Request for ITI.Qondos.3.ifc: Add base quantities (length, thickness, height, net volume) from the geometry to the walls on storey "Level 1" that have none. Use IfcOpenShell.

First a look at what the model holds.

```python
import ifcopenshell
import ifcopenshell.util.element
import ifcopenshell.util.unit

model = ifcopenshell.open("ITI.Qondos.3.ifc")
print(model.schema)
for unit_type in ("LENGTHUNIT", "AREAUNIT", "VOLUMEUNIT"):
    print(unit_type, ifcopenshell.util.unit.calculate_unit_scale(model, unit_type))
storey = next(s for s in model.by_type("IfcBuildingStorey") if s.Name == "Level 1")
walls = [e for e in ifcopenshell.util.element.get_decomposition(storey) if e.is_a("IfcWall")]
for e in sorted(walls, key=lambda e: e.id()):
    print(e.id(), e.is_a(), e.Name, list(ifcopenshell.util.element.get_psets(e, qtos_only=True)), sep=" | ")
```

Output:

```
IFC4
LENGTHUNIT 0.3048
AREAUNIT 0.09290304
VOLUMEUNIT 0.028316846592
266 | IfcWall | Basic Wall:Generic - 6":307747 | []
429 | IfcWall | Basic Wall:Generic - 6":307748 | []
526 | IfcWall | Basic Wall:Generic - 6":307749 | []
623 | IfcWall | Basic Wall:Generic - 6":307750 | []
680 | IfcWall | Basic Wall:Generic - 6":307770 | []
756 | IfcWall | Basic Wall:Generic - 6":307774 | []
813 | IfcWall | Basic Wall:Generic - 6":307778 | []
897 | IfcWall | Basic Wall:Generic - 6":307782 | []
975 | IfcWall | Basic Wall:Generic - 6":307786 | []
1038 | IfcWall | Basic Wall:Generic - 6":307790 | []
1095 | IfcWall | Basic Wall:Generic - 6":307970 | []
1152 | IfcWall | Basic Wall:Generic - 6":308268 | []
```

```python
import ifcopenshell
import ifcopenshell.api.pset
import ifcopenshell.geom
import ifcopenshell.util.element
import ifcopenshell.util.shape
import ifcopenshell.util.unit

model = ifcopenshell.open("ITI.Qondos.3.ifc")
unit_scale = ifcopenshell.util.unit.calculate_unit_scale(model)
volume_scale = ifcopenshell.util.unit.calculate_unit_scale(model, "VOLUMEUNIT")
settings = ifcopenshell.geom.settings()

storey = next(s for s in model.by_type("IfcBuildingStorey") if s.Name == "Level 1")
walls = [e for e in ifcopenshell.util.element.get_decomposition(storey) if e.is_a("IfcWall")]

for e in sorted(walls, key=lambda e: e.id()):
    if ifcopenshell.util.element.get_psets(e, qtos_only=True, should_inherit=False):
        continue
    # Geometry comes back in metres, in the element's own axes.
    shape = ifcopenshell.geom.create_shape(settings, e)
    values = {
        "Length": ifcopenshell.util.shape.get_x(shape.geometry) / unit_scale,
        "Width": ifcopenshell.util.shape.get_y(shape.geometry) / unit_scale,
        "Height": ifcopenshell.util.shape.get_z(shape.geometry) / unit_scale,
        "NetVolume": ifcopenshell.util.shape.get_volume(shape.geometry) / volume_scale,
    }
    qto = ifcopenshell.api.pset.add_qto(model, product=e, name="Qto_WallBaseQuantities")
    ifcopenshell.api.pset.edit_qto(model, qto=qto, properties=values)
    print(e.id(), {k: round(v, 3) for k, v in values.items()})

model.write("ITI.Qondos.3_updated.ifc")
```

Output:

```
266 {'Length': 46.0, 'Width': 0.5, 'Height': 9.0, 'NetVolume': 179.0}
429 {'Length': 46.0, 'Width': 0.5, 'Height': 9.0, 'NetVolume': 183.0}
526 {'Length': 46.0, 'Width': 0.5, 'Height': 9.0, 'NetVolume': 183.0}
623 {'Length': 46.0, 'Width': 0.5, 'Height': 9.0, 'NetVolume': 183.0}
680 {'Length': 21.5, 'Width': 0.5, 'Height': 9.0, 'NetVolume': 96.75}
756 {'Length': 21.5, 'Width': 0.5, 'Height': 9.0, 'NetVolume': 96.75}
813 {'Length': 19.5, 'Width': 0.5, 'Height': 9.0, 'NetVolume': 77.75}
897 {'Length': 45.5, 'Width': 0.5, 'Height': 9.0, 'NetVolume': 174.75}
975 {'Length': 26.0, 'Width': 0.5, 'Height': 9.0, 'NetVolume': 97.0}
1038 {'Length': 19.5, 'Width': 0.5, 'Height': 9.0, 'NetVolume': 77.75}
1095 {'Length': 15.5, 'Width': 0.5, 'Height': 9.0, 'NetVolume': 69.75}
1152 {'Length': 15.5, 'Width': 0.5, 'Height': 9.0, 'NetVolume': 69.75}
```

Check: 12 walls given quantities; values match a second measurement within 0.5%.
